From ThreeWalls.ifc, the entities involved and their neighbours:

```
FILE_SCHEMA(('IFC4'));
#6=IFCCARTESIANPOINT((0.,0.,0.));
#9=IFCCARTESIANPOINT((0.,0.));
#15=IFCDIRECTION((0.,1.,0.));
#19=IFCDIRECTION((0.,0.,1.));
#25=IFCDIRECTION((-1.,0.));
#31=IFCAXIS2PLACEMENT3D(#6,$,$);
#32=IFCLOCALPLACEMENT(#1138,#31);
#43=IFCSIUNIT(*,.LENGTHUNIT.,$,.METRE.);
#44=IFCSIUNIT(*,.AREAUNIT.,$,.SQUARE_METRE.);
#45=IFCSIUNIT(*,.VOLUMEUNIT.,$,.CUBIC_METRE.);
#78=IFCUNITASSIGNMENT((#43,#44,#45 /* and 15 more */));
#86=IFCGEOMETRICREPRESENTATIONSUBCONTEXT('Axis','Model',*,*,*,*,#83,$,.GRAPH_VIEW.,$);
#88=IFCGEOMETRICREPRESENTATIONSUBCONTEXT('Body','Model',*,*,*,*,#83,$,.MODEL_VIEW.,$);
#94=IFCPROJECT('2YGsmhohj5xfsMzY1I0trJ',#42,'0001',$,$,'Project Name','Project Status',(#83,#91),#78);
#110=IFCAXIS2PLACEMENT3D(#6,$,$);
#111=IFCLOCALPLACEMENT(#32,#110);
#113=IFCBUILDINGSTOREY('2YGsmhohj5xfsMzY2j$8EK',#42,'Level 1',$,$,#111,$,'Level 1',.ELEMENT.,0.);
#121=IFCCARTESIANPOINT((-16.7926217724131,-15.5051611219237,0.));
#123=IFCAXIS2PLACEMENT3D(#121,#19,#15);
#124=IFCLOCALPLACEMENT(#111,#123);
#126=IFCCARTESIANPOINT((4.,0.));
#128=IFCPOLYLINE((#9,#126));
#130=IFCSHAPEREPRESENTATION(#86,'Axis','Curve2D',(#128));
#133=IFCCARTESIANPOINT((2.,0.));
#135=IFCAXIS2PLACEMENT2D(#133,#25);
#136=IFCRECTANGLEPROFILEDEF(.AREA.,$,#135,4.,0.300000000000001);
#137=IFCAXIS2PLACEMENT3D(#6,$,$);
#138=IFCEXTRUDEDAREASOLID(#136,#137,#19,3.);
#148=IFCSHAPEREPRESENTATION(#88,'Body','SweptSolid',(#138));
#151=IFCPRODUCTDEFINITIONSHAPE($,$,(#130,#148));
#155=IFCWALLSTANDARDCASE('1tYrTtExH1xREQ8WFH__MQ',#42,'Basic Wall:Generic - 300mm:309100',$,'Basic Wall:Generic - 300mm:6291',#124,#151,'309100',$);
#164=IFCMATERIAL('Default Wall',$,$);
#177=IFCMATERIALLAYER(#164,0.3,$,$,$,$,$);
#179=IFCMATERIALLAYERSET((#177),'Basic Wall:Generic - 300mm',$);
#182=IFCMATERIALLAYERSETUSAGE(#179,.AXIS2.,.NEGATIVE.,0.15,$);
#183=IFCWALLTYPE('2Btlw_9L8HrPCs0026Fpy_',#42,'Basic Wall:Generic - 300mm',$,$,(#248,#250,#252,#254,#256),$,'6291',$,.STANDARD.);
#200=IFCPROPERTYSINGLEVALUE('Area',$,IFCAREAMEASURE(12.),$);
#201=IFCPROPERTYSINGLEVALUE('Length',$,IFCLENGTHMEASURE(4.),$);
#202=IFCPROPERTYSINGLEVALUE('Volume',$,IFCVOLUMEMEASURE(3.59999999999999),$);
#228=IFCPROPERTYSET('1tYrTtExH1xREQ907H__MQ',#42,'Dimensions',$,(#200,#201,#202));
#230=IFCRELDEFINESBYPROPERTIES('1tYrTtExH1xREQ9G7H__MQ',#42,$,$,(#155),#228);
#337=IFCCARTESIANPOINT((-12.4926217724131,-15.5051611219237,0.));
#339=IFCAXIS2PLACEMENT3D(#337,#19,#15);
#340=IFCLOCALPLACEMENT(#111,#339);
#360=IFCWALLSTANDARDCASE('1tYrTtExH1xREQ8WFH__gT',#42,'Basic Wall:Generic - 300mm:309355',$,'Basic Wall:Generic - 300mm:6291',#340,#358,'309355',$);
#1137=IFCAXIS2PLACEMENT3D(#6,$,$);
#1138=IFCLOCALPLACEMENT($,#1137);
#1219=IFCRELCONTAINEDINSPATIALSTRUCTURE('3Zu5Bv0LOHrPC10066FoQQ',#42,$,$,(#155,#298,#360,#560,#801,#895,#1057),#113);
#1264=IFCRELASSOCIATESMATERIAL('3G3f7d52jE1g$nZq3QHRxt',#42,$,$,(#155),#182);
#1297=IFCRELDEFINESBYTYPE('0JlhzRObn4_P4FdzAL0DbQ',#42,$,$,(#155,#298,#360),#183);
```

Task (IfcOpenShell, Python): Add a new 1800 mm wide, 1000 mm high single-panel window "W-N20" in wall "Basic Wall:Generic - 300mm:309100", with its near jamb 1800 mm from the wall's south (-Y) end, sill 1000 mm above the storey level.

```python
import numpy as np
import ifcopenshell
import ifcopenshell.api.feature
import ifcopenshell.api.geometry
import ifcopenshell.api.pset
import ifcopenshell.api.root
import ifcopenshell.api.spatial
import ifcopenshell.geom
import ifcopenshell.util.element
import ifcopenshell.util.placement
import ifcopenshell.util.representation
import ifcopenshell.util.shape
import ifcopenshell.util.unit

model = ifcopenshell.open("ThreeWalls.ifc")
unit_scale = ifcopenshell.util.unit.calculate_unit_scale(model)
area_scale = ifcopenshell.util.unit.calculate_unit_scale(model, "AREAUNIT")
volume_scale = ifcopenshell.util.unit.calculate_unit_scale(model, "VOLUMEUNIT")
settings = ifcopenshell.geom.settings()


def volume(element):
    """Net volume in cubic metres, openings subtracted."""
    shape = ifcopenshell.geom.create_shape(settings, element)
    return ifcopenshell.util.shape.get_volume(shape.geometry)


wall = model.by_guid("1tYrTtExH1xREQ8WFH__MQ")
storey = ifcopenshell.util.element.get_container(wall, ifc_class="IfcBuildingStorey")
context = ifcopenshell.util.representation.get_context(model, "Model", "Body", "MODEL_VIEW")
before = volume(wall)

width, height, from_end, sill = 1.8, 1, 1.8, 1  # metres

# The wall runs along its own X axis, and the end named is its -X end.
wall_shape = ifcopenshell.geom.create_shape(settings, wall)
x, y, z = ifcopenshell.util.shape.get_vertices(wall_shape.geometry).T
start = x.min() + from_end
face, thickness = float(y.min()), float(y.max() - y.min())
wall_matrix = ifcopenshell.util.placement.get_local_placement(wall.ObjectPlacement)
level = ifcopenshell.util.placement.get_local_placement(storey.ObjectPlacement)[2, 3]


def in_wall(x, y):
    """Placement at x, y metres in the wall's axes, at sill height."""
    matrix = wall_matrix.copy()
    matrix[:, 3] = wall_matrix @ np.array([x / unit_scale, y / unit_scale, 0.0, 1.0])
    matrix[2, 3] = level + sill / unit_scale
    return matrix


# Opening: a box that overshoots both wall faces by 50 mm.
opening = ifcopenshell.api.root.create_entity(model, ifc_class="IfcOpeningElement", predefined_type="OPENING")
box = ifcopenshell.api.geometry.add_wall_representation(
    model, context=context, length=width, height=height, thickness=thickness + 0.1
)
ifcopenshell.api.geometry.assign_representation(model, product=opening, representation=box)
ifcopenshell.api.geometry.edit_object_placement(model, product=opening, matrix=in_wall(start, face - 0.05), is_si=False)
ifcopenshell.api.feature.add_feature(model, feature=opening, element=wall)

window = ifcopenshell.api.root.create_entity(model, ifc_class="IfcWindow", name="W-N20", predefined_type="WINDOW")
window.OverallWidth, window.OverallHeight = width / unit_scale, height / unit_scale
window.PartitioningType = "SINGLE_PANEL"
body = ifcopenshell.api.geometry.add_window_representation(
    model,
    context=context,
    overall_width=window.OverallWidth,
    overall_height=window.OverallHeight,
    partition_type="SINGLE_PANEL",
)
ifcopenshell.api.geometry.assign_representation(model, product=window, representation=body)
ifcopenshell.api.spatial.assign_container(model, products=[window], relating_structure=storey)
ifcopenshell.api.feature.add_filling(model, opening=opening, element=window)

# Centre the window in the wall's thickness.
ifcopenshell.api.geometry.edit_object_placement(model, product=window, matrix=in_wall(start, face), is_si=False)
window_shape = ifcopenshell.geom.create_shape(settings, window)
depth = ifcopenshell.util.shape.get_vertices(window_shape.geometry)[:, 1]
offset = face + thickness / 2 - (depth.min() + depth.max()) / 2
ifcopenshell.api.geometry.edit_object_placement(model, product=window, matrix=in_wall(start, offset), is_si=False)

after = volume(wall)

# Update the wall's stored quantities.
pset = model.by_id(ifcopenshell.util.element.get_pset(wall, "Dimensions", should_inherit=False)["id"])
ifcopenshell.api.pset.edit_pset(model, pset=pset, properties={
    "Area": model.create_entity("IfcAreaMeasure", after / thickness / area_scale),
    "Volume": model.create_entity("IfcVolumeMeasure", after / volume_scale),
})

print(f"wall volume {before:.3f} -> {after:.3f} m3")

model.write("ThreeWalls_updated.ifc")
```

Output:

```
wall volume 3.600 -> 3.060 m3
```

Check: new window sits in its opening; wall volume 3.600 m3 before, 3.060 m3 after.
